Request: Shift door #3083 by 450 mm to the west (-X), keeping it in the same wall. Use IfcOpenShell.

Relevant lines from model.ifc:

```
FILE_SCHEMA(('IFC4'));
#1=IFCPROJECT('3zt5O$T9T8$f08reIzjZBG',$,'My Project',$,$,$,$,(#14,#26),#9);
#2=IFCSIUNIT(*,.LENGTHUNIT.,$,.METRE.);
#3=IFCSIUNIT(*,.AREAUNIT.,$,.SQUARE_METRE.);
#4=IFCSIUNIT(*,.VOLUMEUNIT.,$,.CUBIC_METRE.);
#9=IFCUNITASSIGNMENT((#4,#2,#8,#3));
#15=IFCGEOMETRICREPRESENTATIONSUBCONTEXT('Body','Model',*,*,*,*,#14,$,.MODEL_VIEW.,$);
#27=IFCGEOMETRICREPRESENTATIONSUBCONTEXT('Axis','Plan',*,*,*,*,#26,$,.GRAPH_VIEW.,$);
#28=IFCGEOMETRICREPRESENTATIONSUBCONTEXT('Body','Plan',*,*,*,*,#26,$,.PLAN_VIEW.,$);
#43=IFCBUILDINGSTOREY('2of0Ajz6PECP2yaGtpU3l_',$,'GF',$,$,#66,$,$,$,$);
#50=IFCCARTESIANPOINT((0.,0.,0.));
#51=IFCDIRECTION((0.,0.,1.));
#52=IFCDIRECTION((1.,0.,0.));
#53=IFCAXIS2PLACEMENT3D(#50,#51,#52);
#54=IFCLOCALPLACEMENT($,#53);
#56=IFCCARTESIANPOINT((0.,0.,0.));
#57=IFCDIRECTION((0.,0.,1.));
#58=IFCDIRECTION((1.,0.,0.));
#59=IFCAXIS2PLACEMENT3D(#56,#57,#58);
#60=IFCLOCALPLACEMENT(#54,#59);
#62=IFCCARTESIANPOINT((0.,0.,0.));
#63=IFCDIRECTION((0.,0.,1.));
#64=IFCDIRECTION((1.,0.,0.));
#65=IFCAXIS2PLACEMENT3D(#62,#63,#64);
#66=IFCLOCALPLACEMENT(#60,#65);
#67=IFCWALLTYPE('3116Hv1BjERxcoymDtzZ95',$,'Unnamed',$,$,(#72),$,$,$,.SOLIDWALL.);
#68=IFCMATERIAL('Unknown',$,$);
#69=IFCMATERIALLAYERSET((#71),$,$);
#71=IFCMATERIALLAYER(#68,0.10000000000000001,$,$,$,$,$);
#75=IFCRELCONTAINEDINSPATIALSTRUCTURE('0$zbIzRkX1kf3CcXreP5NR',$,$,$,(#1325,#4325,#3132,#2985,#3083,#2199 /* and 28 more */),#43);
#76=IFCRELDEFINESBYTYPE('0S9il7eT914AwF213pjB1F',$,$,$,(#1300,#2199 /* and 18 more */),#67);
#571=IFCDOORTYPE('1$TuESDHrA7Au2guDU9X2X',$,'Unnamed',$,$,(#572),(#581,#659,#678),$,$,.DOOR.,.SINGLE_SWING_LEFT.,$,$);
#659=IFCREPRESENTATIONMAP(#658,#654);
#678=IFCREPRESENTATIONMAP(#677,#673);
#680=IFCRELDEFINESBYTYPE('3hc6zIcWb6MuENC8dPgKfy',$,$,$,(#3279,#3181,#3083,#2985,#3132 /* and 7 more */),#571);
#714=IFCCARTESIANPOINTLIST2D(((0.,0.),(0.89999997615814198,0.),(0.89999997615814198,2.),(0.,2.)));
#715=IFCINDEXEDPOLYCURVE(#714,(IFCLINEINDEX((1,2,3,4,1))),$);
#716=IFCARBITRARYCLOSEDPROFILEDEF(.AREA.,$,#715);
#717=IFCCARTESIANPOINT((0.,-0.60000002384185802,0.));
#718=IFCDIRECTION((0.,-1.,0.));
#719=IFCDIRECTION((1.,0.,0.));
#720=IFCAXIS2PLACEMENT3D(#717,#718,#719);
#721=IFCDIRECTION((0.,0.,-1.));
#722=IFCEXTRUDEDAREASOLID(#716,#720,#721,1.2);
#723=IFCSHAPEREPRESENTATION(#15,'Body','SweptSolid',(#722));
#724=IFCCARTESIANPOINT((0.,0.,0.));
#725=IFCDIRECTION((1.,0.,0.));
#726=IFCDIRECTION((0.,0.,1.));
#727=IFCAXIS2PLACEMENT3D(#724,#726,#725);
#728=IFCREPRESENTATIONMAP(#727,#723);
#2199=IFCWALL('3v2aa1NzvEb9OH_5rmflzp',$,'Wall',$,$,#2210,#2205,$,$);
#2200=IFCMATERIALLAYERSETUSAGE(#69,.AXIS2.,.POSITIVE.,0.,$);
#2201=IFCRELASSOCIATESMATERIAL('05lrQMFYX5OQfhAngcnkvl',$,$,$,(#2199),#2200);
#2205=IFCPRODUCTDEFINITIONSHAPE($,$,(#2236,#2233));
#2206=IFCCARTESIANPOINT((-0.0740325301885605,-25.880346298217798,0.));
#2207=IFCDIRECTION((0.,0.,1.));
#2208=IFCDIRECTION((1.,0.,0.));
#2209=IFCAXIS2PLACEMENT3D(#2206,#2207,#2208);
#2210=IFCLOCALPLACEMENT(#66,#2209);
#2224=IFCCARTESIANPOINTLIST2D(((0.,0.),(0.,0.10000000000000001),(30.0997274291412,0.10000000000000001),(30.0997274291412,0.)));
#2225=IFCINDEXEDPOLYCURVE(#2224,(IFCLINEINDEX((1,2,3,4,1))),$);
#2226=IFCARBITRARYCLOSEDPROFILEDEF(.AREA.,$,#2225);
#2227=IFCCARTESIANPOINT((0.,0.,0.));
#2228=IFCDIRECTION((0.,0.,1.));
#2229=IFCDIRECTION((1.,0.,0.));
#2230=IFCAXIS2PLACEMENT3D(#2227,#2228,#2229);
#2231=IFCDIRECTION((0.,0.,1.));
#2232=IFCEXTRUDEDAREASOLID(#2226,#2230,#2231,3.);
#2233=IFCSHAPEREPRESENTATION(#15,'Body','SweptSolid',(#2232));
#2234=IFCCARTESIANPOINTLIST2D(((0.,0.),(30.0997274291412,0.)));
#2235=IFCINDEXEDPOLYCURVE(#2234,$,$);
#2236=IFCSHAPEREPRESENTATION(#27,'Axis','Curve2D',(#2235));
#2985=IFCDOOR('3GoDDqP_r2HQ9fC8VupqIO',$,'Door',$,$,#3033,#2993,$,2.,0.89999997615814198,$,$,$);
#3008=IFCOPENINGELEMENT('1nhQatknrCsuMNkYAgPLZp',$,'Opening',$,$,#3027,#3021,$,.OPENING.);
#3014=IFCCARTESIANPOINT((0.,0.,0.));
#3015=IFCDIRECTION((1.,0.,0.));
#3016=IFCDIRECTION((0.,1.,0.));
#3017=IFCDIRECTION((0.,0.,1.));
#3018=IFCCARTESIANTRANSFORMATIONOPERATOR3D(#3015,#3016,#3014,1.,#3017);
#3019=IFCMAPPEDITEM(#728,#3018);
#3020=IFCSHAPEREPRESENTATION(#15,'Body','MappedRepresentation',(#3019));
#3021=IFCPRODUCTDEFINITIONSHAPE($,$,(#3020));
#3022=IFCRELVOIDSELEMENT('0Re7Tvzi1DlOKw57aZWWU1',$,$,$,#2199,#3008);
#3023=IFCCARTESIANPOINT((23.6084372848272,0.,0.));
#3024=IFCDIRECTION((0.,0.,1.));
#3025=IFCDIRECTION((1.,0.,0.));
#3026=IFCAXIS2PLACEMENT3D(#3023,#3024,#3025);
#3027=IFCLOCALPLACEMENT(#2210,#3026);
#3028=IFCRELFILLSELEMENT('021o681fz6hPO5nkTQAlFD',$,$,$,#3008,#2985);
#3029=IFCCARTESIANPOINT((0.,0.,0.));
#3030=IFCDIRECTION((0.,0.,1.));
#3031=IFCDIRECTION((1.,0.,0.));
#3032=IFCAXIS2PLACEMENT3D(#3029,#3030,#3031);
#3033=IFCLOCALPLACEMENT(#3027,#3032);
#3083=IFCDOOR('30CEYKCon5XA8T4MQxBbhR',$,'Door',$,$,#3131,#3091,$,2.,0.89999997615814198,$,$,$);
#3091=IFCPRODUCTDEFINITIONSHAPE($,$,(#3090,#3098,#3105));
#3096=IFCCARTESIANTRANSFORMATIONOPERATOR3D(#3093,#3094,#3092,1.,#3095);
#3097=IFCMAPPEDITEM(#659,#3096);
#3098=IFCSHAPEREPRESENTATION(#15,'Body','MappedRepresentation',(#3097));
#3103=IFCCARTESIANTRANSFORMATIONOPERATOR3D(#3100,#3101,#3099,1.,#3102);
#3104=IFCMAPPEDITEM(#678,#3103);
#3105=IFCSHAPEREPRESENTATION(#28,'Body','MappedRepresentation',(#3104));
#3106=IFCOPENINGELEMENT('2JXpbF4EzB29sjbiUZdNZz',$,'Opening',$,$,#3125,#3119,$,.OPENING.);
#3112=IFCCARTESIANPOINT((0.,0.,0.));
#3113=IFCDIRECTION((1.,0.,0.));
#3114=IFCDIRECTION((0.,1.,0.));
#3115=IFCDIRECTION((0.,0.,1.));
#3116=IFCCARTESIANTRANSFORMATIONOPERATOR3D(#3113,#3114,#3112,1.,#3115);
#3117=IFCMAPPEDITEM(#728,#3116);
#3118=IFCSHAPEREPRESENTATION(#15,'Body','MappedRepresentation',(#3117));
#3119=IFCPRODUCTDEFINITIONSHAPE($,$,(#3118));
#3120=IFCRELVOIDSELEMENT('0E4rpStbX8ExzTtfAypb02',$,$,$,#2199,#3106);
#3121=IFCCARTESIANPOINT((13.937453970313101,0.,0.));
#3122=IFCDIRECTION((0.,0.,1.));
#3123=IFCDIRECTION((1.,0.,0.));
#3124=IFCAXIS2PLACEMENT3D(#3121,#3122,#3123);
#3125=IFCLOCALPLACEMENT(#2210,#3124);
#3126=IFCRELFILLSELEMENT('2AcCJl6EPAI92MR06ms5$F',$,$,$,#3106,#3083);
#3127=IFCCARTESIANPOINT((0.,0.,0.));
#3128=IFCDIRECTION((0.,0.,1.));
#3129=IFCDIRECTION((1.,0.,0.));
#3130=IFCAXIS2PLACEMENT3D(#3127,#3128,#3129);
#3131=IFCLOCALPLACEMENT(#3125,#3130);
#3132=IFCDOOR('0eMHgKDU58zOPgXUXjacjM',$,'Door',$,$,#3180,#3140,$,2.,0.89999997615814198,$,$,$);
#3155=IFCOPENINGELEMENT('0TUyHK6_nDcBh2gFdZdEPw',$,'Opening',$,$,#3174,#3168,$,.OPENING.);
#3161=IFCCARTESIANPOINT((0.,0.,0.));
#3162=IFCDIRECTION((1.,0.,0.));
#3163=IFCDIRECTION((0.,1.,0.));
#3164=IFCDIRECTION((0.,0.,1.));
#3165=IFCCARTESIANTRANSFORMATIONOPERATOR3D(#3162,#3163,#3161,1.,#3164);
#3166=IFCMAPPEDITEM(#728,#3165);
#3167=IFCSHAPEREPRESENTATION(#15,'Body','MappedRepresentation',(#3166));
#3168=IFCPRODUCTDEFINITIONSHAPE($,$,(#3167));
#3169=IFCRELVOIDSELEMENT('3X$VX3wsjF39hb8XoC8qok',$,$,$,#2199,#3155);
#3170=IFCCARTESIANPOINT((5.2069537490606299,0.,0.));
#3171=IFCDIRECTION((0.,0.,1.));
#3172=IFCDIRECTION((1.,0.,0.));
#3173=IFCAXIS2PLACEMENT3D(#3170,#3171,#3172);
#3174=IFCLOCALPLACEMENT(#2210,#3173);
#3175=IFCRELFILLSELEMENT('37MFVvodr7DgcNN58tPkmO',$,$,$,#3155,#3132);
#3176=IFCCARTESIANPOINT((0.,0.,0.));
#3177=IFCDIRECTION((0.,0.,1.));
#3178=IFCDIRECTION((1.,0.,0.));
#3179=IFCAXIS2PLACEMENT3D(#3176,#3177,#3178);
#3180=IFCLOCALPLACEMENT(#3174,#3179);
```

```python
import ifcopenshell
import ifcopenshell.api.geometry
import ifcopenshell.util.placement
import ifcopenshell.util.unit

model = ifcopenshell.open("model.ifc")
unit_scale = ifcopenshell.util.unit.calculate_unit_scale(model)

door = model.by_guid("30CEYKCon5XA8T4MQxBbhR")
opening = door.FillsVoids[0].RelatingOpeningElement
wall = opening.VoidsElements[0].RelatingBuildingElement

wall_matrix = ifcopenshell.util.placement.get_local_placement(wall.ObjectPlacement)
shift = wall_matrix[:3, 0] * -0.45 / unit_scale
before = ifcopenshell.util.placement.get_local_placement(door.ObjectPlacement)[:3, 3].copy()

# The door is placed relative to its opening, so it follows when the opening moves.
matrix = ifcopenshell.util.placement.get_local_placement(opening.ObjectPlacement)
matrix[:3, 3] += shift
ifcopenshell.api.geometry.edit_object_placement(
    model, product=opening, matrix=matrix, is_si=False, should_transform_children=True
)

after = ifcopenshell.util.placement.get_local_placement(door.ObjectPlacement)[:3, 3]
print("door moved by", (after - before).round(3) + 0.0)

model.write("model_edited.ifc")
```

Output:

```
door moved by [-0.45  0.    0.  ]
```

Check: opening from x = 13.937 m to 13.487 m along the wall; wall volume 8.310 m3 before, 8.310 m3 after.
